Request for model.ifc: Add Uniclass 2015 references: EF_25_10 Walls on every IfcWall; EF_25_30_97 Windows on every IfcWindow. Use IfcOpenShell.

First a look at what the model holds.

```python
import ifcopenshell

model = ifcopenshell.open("model.ifc")
print(model.schema)
print("classifications:", [c.Name for c in model.by_type("IfcClassification")])
for ifc_class in ("IfcDoor", "IfcRoof", "IfcStair", "IfcWall", "IfcWindow"):
    print(ifc_class, len(model.by_type(ifc_class)))
```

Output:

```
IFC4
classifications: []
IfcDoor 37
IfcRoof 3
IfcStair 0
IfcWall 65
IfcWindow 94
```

```python
import ifcopenshell
import ifcopenshell.api.classification

model = ifcopenshell.open("model.ifc")

system = ifcopenshell.api.classification.add_classification(model, classification="Uniclass 2015")

codes = {
    "IfcWall": ("EF_25_10", "Walls"),
    "IfcWindow": ("EF_25_30_97", "Windows"),
}
for ifc_class, (code, name) in codes.items():
    products = model.by_type(ifc_class)
    ifcopenshell.api.classification.add_reference(
        model, products=products, classification=system, identification=code, name=name
    )
    print(code, len(products))

model.write("model_v2.ifc")
```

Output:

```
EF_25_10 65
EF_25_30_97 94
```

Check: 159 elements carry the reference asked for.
